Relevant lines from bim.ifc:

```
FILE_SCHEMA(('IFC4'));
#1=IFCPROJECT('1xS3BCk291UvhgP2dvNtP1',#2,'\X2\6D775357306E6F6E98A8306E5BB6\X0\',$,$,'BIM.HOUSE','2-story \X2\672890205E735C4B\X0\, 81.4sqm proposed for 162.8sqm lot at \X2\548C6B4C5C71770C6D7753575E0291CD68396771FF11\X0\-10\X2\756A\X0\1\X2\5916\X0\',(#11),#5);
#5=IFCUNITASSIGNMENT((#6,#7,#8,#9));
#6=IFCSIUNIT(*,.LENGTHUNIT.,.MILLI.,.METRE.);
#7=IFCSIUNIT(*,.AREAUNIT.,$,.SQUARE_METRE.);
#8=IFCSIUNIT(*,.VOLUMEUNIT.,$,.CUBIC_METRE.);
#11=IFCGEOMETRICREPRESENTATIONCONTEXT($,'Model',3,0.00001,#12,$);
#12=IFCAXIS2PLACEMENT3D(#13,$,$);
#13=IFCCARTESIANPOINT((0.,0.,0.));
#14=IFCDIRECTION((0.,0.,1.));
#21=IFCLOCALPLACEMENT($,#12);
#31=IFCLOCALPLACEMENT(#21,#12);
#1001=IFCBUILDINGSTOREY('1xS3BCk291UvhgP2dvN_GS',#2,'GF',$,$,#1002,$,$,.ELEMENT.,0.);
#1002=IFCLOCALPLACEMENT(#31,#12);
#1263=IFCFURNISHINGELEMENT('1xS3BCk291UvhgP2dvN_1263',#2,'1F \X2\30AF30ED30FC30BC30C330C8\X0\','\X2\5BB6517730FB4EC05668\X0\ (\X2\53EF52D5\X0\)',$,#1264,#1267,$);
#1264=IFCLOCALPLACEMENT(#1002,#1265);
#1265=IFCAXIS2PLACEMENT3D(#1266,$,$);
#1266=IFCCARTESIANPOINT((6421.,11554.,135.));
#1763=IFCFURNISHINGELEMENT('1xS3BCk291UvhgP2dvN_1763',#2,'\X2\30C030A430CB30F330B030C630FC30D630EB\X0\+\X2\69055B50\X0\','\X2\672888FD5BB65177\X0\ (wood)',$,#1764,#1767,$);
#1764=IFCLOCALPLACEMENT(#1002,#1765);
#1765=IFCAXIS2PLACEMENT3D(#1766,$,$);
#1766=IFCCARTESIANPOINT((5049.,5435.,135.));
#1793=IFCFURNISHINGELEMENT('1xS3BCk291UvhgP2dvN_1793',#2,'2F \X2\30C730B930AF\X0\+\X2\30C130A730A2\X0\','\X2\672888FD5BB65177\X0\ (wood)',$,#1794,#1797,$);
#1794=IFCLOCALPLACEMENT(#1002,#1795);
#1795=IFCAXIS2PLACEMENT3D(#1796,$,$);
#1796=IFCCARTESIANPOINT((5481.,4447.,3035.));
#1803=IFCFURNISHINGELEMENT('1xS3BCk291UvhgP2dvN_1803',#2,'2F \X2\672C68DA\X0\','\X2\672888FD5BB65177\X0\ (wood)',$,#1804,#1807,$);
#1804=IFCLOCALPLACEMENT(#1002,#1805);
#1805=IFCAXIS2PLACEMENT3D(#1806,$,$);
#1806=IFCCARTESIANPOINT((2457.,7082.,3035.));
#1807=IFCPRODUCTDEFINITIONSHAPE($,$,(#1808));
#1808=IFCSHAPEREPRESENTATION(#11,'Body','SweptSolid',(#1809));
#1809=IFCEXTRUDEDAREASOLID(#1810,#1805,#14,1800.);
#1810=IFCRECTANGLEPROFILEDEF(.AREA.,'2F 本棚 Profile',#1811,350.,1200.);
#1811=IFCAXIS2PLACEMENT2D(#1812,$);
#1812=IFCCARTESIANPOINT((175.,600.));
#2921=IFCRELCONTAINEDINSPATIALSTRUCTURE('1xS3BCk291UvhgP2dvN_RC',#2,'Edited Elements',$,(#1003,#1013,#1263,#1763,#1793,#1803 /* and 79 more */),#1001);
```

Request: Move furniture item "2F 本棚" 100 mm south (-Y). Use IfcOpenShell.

```python
import ifcopenshell
import ifcopenshell.api.geometry
import ifcopenshell.util.placement
import ifcopenshell.util.unit

model = ifcopenshell.open("bim.ifc")
unit_scale = ifcopenshell.util.unit.calculate_unit_scale(model)

item = model.by_guid("1xS3BCk291UvhgP2dvN_1803")
matrix = ifcopenshell.util.placement.get_local_placement(item.ObjectPlacement)
matrix[1, 3] -= 0.1 / unit_scale
ifcopenshell.api.geometry.edit_object_placement(model, product=item, matrix=matrix, is_si=False)

print(ifcopenshell.util.placement.get_local_placement(item.ObjectPlacement).round(3) + 0.0)

model.write("bim_v2.ifc")
```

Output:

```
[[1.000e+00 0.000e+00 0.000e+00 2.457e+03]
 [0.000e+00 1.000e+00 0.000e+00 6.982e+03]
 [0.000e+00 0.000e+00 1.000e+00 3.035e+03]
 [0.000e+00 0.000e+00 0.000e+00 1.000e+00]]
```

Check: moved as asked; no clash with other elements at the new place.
